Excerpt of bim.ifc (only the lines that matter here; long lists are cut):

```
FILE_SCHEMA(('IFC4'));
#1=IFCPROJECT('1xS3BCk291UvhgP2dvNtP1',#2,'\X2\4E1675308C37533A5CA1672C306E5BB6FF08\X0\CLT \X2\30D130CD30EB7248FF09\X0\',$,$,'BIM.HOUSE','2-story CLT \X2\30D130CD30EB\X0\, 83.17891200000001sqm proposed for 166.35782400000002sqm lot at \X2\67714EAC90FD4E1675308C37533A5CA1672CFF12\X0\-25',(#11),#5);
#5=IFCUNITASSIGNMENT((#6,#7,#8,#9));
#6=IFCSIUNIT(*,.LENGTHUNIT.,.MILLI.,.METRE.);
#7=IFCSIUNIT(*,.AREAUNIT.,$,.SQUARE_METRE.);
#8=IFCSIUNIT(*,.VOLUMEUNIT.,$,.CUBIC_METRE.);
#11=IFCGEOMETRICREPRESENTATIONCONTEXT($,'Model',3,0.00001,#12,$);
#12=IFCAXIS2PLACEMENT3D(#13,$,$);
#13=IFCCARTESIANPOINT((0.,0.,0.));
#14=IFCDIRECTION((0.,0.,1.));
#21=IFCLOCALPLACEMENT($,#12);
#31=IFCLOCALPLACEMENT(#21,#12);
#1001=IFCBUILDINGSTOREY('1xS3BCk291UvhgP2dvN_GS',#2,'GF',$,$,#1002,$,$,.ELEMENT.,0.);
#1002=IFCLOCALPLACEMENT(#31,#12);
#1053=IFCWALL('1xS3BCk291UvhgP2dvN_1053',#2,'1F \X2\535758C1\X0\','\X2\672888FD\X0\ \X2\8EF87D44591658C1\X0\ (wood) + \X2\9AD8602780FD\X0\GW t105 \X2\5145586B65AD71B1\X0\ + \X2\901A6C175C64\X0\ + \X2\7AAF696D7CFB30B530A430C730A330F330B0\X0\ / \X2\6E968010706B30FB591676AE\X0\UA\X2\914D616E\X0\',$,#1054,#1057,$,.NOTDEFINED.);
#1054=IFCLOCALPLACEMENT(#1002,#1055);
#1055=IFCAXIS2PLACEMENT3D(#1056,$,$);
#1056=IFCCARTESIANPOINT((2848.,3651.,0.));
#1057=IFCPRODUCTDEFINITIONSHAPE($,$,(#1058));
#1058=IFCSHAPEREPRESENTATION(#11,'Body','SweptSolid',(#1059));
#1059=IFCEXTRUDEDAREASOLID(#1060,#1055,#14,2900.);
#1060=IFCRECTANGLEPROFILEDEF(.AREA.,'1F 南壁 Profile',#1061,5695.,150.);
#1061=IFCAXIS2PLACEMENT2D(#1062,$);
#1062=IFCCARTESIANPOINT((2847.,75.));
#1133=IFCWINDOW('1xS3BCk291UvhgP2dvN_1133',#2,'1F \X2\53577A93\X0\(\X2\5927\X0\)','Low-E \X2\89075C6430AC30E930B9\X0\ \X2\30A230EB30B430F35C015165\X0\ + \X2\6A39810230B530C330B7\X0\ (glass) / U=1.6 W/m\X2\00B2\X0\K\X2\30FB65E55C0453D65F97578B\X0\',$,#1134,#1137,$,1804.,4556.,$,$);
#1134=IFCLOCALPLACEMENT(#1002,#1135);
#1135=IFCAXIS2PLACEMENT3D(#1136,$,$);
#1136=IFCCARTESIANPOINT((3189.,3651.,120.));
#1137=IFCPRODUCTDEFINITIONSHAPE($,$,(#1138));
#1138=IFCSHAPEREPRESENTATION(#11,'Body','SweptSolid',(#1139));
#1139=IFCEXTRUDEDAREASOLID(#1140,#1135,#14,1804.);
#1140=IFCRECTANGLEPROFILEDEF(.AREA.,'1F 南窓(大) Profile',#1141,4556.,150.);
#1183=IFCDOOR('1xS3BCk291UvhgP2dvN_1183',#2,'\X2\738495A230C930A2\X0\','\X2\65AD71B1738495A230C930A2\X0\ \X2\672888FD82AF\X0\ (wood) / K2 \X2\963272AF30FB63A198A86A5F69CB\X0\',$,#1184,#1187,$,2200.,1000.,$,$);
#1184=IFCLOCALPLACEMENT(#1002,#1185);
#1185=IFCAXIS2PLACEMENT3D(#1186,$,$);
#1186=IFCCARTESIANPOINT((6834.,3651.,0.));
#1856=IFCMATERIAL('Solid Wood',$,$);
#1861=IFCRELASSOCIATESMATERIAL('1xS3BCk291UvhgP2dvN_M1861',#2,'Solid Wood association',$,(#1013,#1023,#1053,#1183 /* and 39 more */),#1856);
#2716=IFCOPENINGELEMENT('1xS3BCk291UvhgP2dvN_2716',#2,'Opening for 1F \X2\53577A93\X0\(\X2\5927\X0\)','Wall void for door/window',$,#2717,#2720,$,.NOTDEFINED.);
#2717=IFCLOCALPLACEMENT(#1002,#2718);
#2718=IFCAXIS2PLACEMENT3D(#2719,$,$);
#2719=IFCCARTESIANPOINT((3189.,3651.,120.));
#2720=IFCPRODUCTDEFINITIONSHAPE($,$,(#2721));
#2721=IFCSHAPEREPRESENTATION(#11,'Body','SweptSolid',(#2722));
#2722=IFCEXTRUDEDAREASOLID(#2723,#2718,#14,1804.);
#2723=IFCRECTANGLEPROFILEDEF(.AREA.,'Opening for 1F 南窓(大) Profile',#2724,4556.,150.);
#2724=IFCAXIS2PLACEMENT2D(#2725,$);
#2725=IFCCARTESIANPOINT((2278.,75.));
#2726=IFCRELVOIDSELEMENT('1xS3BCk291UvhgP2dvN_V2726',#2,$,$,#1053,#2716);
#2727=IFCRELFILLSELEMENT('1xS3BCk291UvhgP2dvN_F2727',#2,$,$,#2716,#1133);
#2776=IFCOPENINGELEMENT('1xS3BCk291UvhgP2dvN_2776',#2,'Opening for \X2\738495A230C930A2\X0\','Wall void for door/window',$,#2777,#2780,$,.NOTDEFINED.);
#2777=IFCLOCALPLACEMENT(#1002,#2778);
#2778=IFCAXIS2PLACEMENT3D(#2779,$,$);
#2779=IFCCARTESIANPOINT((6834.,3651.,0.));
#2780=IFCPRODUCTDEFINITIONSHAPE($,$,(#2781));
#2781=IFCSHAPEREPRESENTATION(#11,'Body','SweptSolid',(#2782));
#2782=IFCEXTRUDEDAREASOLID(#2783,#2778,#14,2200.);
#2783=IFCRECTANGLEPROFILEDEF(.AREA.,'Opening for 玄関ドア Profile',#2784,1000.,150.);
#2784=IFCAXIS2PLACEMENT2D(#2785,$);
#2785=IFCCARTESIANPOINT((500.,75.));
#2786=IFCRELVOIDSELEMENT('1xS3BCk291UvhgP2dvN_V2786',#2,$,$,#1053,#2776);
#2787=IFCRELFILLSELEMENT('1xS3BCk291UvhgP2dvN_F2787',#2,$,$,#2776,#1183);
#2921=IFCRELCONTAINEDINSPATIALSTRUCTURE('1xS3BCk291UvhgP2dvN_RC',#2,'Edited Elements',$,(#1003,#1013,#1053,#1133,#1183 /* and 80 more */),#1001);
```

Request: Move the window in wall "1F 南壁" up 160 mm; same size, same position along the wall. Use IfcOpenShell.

```python
import numpy as np
import ifcopenshell
import ifcopenshell.api.geometry
import ifcopenshell.util.placement
import ifcopenshell.util.unit

model = ifcopenshell.open("bim.ifc")
unit_scale = ifcopenshell.util.unit.calculate_unit_scale(model)

window = model.by_id(1133)
opening = window.FillsVoids[0].RelatingOpeningElement
dz = 160.0

shift = np.array([0.0, 0.0, dz])
# The window is not placed relative to its opening, so move both.
for product in (opening, window):
    matrix = ifcopenshell.util.placement.get_local_placement(product.ObjectPlacement)
    matrix[:3, 3] += shift
    ifcopenshell.api.geometry.edit_object_placement(model, product=product, matrix=matrix, is_si=False)

print(f"moved by {dz * unit_scale:+.3f} m")

model.write("bim_v2.ifc")
```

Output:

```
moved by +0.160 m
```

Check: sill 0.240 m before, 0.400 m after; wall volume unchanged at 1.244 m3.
